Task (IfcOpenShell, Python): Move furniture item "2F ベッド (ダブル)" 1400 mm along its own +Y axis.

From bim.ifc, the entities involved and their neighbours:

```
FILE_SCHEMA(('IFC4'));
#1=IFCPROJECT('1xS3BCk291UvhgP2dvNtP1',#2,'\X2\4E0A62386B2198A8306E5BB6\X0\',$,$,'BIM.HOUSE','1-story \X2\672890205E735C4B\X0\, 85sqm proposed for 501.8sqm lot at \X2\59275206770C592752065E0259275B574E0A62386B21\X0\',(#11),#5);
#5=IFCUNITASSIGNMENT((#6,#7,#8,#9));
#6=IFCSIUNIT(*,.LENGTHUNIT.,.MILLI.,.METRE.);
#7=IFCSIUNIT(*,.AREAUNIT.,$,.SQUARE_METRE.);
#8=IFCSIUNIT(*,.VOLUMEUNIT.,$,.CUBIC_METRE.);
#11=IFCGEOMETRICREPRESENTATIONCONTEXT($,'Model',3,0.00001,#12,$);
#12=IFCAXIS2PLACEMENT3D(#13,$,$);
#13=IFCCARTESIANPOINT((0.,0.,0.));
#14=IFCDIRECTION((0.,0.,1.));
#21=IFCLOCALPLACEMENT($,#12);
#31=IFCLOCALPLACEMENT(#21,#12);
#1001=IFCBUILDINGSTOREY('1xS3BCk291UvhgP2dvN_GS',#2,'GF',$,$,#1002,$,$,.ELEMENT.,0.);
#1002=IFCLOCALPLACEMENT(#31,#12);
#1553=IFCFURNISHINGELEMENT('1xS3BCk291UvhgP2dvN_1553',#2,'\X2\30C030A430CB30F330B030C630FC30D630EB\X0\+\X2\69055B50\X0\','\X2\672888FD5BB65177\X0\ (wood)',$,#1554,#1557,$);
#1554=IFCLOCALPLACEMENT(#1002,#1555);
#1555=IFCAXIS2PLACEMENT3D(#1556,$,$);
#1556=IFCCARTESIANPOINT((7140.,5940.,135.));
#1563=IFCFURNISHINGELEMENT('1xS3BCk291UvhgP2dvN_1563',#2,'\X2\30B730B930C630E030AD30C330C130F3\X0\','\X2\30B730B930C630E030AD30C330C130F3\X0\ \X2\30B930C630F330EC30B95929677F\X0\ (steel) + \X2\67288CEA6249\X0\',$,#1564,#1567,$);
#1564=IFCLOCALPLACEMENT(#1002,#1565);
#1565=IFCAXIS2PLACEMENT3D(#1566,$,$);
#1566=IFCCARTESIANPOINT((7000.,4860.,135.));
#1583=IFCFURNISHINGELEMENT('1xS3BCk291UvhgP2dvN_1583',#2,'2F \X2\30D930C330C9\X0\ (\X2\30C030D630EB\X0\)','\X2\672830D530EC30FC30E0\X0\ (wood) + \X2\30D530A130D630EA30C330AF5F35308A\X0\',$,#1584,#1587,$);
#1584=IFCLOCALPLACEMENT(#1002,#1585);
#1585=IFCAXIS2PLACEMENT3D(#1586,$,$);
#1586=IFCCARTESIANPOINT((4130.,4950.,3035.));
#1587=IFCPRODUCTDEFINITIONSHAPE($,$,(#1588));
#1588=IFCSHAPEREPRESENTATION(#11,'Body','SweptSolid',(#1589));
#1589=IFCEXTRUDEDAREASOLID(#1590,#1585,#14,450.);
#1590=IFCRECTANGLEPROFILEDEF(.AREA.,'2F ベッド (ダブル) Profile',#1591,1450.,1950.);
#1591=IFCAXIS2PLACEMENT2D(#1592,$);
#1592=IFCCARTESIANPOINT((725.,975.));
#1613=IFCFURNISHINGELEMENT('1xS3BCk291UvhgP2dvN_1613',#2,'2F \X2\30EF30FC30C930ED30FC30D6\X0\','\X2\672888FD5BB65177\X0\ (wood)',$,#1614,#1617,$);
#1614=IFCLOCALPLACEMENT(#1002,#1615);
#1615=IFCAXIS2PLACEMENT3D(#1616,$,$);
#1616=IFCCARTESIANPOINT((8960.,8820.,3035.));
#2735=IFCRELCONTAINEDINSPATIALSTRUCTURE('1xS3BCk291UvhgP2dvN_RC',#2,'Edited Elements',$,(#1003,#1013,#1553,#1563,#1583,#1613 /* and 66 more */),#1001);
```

```python
import ifcopenshell
import ifcopenshell.api.geometry
import ifcopenshell.util.placement
import ifcopenshell.util.unit

model = ifcopenshell.open("bim.ifc")
unit_scale = ifcopenshell.util.unit.calculate_unit_scale(model)

item = model.by_guid("1xS3BCk291UvhgP2dvN_1583")
matrix = ifcopenshell.util.placement.get_local_placement(item.ObjectPlacement)
matrix[:3, 3] += matrix[:3, 1] * 1.4 / unit_scale
ifcopenshell.api.geometry.edit_object_placement(model, product=item, matrix=matrix, is_si=False)

print(ifcopenshell.util.placement.get_local_placement(item.ObjectPlacement).round(3) + 0.0)

model.write("bim-out.ifc")
```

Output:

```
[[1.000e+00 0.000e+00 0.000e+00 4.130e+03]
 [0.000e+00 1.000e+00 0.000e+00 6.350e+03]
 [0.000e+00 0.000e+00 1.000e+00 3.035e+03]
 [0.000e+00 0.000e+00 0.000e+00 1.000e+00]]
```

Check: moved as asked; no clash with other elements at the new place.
